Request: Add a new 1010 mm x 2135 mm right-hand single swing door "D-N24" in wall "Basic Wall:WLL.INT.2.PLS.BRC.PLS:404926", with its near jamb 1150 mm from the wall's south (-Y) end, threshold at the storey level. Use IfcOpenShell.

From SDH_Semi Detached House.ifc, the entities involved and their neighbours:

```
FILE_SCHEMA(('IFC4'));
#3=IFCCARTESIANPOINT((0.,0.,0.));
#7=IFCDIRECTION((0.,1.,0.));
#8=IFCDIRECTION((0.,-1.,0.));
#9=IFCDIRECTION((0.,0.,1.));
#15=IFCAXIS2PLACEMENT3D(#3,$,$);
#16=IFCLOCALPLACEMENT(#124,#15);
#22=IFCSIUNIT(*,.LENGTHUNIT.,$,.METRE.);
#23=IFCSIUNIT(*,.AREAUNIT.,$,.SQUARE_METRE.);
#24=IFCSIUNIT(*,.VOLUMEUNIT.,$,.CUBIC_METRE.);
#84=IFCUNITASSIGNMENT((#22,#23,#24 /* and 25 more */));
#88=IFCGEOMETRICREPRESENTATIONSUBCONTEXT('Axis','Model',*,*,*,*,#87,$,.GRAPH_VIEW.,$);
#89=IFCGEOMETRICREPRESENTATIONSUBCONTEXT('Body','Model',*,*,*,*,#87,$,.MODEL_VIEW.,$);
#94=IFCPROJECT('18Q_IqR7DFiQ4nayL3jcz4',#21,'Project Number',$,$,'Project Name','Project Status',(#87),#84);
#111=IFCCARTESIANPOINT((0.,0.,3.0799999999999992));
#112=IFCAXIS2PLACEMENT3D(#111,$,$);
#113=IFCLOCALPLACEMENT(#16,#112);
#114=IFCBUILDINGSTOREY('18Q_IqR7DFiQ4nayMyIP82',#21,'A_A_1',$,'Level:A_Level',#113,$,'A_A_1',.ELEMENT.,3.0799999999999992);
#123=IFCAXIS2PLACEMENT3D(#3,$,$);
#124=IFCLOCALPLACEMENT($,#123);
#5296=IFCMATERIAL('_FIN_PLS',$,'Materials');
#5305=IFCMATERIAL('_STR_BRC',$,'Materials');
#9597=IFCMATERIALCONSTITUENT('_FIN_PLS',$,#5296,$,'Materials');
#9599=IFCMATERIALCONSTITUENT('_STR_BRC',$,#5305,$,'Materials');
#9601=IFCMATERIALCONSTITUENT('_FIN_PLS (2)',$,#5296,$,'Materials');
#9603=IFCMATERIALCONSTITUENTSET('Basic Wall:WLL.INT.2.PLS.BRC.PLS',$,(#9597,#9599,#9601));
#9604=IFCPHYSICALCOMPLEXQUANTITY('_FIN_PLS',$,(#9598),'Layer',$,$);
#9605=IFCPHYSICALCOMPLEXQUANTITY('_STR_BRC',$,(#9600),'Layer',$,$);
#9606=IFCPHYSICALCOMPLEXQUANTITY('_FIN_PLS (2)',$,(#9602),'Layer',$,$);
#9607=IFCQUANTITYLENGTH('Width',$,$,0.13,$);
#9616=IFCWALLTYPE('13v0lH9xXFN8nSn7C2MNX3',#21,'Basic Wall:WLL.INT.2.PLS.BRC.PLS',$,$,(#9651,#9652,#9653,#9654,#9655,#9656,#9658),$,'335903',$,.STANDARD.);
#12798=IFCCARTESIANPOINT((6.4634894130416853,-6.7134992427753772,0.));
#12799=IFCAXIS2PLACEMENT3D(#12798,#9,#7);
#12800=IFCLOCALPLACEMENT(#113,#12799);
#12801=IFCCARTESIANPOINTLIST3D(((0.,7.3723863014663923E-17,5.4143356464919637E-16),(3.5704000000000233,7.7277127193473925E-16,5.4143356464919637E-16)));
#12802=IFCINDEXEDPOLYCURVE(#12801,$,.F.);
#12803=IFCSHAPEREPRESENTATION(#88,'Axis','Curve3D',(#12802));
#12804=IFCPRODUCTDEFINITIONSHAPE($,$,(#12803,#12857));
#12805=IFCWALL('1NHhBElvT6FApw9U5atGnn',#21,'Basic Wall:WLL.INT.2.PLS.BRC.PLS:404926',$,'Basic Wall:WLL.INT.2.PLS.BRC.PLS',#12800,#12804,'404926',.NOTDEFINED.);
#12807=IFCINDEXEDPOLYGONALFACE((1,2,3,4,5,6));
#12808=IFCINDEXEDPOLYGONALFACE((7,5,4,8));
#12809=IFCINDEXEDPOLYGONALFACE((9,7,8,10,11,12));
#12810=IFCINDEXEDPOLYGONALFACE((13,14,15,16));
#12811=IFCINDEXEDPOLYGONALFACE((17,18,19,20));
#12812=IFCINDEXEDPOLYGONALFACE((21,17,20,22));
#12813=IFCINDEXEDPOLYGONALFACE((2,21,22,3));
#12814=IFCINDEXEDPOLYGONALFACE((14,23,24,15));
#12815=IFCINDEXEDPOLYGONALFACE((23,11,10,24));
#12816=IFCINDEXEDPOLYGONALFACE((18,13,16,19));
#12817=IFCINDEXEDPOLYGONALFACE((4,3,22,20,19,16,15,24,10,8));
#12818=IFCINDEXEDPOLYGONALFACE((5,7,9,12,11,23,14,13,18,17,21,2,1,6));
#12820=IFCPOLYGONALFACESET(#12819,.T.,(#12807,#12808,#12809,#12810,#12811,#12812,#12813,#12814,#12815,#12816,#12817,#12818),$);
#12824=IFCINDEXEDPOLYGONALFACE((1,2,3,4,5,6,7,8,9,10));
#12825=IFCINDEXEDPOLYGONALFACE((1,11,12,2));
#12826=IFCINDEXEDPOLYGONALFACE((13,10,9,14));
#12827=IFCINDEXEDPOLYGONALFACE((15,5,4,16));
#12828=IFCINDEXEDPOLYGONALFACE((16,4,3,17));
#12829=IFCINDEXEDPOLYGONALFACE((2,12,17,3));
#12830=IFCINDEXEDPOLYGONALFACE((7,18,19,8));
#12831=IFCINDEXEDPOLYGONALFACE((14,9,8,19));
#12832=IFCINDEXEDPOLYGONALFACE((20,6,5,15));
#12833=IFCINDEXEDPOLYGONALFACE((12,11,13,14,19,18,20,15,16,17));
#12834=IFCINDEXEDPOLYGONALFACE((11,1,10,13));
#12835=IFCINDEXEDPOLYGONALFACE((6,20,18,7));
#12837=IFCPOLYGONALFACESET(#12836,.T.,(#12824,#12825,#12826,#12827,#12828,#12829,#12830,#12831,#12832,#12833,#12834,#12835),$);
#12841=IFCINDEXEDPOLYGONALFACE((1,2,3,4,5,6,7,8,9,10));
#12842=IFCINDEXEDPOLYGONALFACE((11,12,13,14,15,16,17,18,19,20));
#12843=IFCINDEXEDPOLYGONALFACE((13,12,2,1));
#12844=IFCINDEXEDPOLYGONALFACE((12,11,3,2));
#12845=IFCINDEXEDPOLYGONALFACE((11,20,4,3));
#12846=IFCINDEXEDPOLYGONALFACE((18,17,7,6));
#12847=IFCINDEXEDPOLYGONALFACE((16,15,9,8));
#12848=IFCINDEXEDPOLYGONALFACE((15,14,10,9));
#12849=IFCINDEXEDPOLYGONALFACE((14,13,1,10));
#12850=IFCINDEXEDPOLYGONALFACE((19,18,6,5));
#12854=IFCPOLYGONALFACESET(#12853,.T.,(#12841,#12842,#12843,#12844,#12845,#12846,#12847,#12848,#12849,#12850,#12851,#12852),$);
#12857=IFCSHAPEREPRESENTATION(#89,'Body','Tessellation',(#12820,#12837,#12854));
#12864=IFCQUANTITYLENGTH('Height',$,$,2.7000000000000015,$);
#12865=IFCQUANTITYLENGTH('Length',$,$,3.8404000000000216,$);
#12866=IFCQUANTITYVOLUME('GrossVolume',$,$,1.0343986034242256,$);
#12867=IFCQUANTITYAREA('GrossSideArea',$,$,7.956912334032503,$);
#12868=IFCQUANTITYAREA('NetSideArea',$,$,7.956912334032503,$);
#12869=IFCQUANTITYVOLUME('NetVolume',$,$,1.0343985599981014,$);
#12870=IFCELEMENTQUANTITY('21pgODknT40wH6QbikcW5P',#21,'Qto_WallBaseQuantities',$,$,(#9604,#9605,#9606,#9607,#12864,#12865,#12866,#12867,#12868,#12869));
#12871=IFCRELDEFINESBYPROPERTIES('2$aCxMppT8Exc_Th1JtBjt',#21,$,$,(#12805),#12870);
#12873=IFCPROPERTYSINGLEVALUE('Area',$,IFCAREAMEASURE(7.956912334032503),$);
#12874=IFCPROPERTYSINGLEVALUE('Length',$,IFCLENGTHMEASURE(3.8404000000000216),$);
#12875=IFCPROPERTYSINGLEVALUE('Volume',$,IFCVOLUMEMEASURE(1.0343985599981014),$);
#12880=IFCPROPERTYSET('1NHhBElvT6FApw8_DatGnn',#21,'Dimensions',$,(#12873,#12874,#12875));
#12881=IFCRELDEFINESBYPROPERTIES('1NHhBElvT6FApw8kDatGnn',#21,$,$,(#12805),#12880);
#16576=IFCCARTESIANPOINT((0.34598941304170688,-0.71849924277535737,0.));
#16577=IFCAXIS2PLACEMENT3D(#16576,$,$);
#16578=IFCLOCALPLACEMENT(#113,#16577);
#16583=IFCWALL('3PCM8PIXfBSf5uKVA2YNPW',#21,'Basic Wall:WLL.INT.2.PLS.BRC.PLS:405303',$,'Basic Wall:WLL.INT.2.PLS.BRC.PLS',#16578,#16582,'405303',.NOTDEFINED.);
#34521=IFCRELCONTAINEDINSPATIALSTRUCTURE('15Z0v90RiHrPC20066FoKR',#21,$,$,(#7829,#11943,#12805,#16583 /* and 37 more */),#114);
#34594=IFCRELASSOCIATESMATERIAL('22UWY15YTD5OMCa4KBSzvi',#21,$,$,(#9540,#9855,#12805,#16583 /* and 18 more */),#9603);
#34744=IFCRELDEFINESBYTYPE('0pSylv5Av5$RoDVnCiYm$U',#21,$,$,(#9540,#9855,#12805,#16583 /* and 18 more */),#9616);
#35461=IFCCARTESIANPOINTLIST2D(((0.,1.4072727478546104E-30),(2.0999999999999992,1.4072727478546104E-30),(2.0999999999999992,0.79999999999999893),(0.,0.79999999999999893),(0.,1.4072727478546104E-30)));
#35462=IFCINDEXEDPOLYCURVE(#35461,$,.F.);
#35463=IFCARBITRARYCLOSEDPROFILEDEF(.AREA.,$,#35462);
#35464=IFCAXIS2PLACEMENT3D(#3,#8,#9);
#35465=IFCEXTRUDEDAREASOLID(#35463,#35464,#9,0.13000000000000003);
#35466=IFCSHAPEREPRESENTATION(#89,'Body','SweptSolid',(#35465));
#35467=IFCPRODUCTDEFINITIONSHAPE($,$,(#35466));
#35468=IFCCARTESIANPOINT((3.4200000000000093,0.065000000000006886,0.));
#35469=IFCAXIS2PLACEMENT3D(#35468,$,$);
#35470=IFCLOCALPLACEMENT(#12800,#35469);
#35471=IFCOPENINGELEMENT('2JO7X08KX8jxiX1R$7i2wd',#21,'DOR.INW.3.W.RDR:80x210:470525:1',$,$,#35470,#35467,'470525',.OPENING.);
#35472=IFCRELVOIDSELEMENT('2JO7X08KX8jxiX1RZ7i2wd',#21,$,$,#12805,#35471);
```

```python
import numpy as np
import ifcopenshell
import ifcopenshell.api.feature
import ifcopenshell.api.geometry
import ifcopenshell.api.pset
import ifcopenshell.api.root
import ifcopenshell.api.spatial
import ifcopenshell.geom
import ifcopenshell.util.element
import ifcopenshell.util.placement
import ifcopenshell.util.representation
import ifcopenshell.util.shape
import ifcopenshell.util.unit

model = ifcopenshell.open("SDH_Semi Detached House.ifc")
unit_scale = ifcopenshell.util.unit.calculate_unit_scale(model)
area_scale = ifcopenshell.util.unit.calculate_unit_scale(model, "AREAUNIT")
volume_scale = ifcopenshell.util.unit.calculate_unit_scale(model, "VOLUMEUNIT")
settings = ifcopenshell.geom.settings()


def volume(element):
    """Net volume in cubic metres, openings subtracted."""
    shape = ifcopenshell.geom.create_shape(settings, element)
    return ifcopenshell.util.shape.get_volume(shape.geometry)


wall = model.by_guid("1NHhBElvT6FApw9U5atGnn")
storey = ifcopenshell.util.element.get_container(wall, ifc_class="IfcBuildingStorey")
context = ifcopenshell.util.representation.get_context(model, "Model", "Body", "MODEL_VIEW")
before = volume(wall)

width, height, from_end, sill = 1.01, 2.135, 1.15, 0.0  # metres

# The wall runs along its own X axis, and the end named is its -X end.
wall_shape = ifcopenshell.geom.create_shape(settings, wall)
x, y, z = ifcopenshell.util.shape.get_vertices(wall_shape.geometry).T
start = x.min() + from_end
face, thickness = float(y.min()), float(y.max() - y.min())
wall_matrix = ifcopenshell.util.placement.get_local_placement(wall.ObjectPlacement)
level = ifcopenshell.util.placement.get_local_placement(storey.ObjectPlacement)[2, 3]


def in_wall(x, y):
    """Placement at x, y metres in the wall's axes, at sill height."""
    matrix = wall_matrix.copy()
    matrix[:, 3] = wall_matrix @ np.array([x / unit_scale, y / unit_scale, 0.0, 1.0])
    matrix[2, 3] = level + sill / unit_scale
    return matrix


# Opening: a box that overshoots both wall faces by 50 mm.
opening = ifcopenshell.api.root.create_entity(model, ifc_class="IfcOpeningElement", predefined_type="OPENING")
box = ifcopenshell.api.geometry.add_wall_representation(
    model, context=context, length=width, height=height, thickness=thickness + 0.1
)
ifcopenshell.api.geometry.assign_representation(model, product=opening, representation=box)
ifcopenshell.api.geometry.edit_object_placement(model, product=opening, matrix=in_wall(start, face - 0.05), is_si=False)
ifcopenshell.api.feature.add_feature(model, feature=opening, element=wall)

door = ifcopenshell.api.root.create_entity(model, ifc_class="IfcDoor", name="D-N24", predefined_type="DOOR")
door.OverallWidth, door.OverallHeight = width / unit_scale, height / unit_scale
door.OperationType = "SINGLE_SWING_RIGHT"
body = ifcopenshell.api.geometry.add_door_representation(
    model,
    context=context,
    overall_width=door.OverallWidth,
    overall_height=door.OverallHeight,
    operation_type="SINGLE_SWING_RIGHT",
    lining_properties={"LiningDepth": thickness / unit_scale, "ThresholdDepth": thickness / unit_scale},
)
ifcopenshell.api.geometry.assign_representation(model, product=door, representation=body)
ifcopenshell.api.spatial.assign_container(model, products=[door], relating_structure=storey)
ifcopenshell.api.feature.add_filling(model, opening=opening, element=door)

# The lining spans the wall, so the door starts at the wall face.
ifcopenshell.api.geometry.edit_object_placement(model, product=door, matrix=in_wall(start, face), is_si=False)

after = volume(wall)

# Update the wall's stored quantities.
qto = model.by_id(ifcopenshell.util.element.get_pset(wall, "Qto_WallBaseQuantities", should_inherit=False)["id"])
ifcopenshell.api.pset.edit_qto(model, qto=qto, properties={
    "NetSideArea": after / thickness / area_scale,
    "NetVolume": after / volume_scale,
})
pset = model.by_id(ifcopenshell.util.element.get_pset(wall, "Dimensions", should_inherit=False)["id"])
ifcopenshell.api.pset.edit_pset(model, pset=pset, properties={
    "Area": model.create_entity("IfcAreaMeasure", after / thickness / area_scale),
    "Volume": model.create_entity("IfcVolumeMeasure", after / volume_scale),
})

print(f"wall volume {before:.3f} -> {after:.3f} m3")

model.write("SDH_Semi Detached House_rev.ifc")
```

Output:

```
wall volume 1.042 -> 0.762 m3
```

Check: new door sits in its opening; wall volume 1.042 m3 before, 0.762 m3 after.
